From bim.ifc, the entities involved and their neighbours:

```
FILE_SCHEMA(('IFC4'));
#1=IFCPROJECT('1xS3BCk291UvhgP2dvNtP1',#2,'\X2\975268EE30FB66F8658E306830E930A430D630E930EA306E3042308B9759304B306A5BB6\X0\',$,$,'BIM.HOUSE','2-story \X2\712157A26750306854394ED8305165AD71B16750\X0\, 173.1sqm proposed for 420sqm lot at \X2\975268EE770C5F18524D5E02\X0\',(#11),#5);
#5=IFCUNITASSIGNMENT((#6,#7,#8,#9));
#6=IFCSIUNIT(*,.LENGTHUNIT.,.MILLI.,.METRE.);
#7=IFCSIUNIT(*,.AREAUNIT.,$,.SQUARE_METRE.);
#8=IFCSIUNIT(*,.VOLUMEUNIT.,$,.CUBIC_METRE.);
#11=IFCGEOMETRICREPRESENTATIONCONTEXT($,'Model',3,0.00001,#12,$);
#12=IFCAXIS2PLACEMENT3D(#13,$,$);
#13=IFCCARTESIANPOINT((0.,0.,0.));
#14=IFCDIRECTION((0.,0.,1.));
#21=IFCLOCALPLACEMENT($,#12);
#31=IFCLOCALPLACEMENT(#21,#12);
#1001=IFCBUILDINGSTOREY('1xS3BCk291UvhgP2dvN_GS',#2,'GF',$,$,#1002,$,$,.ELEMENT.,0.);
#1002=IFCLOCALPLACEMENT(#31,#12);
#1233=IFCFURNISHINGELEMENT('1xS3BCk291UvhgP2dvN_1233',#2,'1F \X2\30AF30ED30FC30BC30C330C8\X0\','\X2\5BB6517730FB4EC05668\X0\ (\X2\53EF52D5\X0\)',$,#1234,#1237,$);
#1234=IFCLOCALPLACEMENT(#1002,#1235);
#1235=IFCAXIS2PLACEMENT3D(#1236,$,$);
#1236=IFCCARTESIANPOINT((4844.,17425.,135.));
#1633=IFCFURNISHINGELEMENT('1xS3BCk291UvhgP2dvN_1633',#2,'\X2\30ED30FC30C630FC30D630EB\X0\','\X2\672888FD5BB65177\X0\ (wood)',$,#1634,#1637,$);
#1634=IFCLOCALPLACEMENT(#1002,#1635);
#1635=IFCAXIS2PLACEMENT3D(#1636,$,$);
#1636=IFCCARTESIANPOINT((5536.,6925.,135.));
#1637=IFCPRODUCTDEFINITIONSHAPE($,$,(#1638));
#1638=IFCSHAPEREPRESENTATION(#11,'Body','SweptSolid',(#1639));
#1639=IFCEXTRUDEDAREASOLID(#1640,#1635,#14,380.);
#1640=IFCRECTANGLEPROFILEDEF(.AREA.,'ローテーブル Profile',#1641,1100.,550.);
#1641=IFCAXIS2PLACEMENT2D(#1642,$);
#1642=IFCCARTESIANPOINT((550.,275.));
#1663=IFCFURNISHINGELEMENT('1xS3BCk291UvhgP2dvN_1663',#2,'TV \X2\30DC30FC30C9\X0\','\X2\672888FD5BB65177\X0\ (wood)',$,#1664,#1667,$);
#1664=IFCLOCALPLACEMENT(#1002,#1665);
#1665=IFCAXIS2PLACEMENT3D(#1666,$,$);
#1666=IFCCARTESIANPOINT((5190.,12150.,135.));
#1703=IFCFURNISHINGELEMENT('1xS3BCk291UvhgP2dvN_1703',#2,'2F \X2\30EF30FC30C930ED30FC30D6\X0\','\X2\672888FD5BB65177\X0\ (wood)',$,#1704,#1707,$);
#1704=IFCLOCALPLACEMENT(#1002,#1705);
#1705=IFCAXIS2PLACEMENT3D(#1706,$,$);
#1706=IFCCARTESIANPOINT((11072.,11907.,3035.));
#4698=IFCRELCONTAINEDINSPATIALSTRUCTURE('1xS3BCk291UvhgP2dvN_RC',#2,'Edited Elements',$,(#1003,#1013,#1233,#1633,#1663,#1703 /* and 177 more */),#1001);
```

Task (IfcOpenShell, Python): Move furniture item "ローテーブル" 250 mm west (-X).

```python
import ifcopenshell
import ifcopenshell.api.geometry
import ifcopenshell.util.placement

model = ifcopenshell.open("bim.ifc")

item = model.by_guid("1xS3BCk291UvhgP2dvN_1633")
matrix = ifcopenshell.util.placement.get_local_placement(item.ObjectPlacement)
matrix[0, 3] -= 250.0
ifcopenshell.api.geometry.edit_object_placement(model, product=item, matrix=matrix, is_si=False)

print(ifcopenshell.util.placement.get_local_placement(item.ObjectPlacement).round(3) + 0.0)

model.write("bim_rev.ifc")
```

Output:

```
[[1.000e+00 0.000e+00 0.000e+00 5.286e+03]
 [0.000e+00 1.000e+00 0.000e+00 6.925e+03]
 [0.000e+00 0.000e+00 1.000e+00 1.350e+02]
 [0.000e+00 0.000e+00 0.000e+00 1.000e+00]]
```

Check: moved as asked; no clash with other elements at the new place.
